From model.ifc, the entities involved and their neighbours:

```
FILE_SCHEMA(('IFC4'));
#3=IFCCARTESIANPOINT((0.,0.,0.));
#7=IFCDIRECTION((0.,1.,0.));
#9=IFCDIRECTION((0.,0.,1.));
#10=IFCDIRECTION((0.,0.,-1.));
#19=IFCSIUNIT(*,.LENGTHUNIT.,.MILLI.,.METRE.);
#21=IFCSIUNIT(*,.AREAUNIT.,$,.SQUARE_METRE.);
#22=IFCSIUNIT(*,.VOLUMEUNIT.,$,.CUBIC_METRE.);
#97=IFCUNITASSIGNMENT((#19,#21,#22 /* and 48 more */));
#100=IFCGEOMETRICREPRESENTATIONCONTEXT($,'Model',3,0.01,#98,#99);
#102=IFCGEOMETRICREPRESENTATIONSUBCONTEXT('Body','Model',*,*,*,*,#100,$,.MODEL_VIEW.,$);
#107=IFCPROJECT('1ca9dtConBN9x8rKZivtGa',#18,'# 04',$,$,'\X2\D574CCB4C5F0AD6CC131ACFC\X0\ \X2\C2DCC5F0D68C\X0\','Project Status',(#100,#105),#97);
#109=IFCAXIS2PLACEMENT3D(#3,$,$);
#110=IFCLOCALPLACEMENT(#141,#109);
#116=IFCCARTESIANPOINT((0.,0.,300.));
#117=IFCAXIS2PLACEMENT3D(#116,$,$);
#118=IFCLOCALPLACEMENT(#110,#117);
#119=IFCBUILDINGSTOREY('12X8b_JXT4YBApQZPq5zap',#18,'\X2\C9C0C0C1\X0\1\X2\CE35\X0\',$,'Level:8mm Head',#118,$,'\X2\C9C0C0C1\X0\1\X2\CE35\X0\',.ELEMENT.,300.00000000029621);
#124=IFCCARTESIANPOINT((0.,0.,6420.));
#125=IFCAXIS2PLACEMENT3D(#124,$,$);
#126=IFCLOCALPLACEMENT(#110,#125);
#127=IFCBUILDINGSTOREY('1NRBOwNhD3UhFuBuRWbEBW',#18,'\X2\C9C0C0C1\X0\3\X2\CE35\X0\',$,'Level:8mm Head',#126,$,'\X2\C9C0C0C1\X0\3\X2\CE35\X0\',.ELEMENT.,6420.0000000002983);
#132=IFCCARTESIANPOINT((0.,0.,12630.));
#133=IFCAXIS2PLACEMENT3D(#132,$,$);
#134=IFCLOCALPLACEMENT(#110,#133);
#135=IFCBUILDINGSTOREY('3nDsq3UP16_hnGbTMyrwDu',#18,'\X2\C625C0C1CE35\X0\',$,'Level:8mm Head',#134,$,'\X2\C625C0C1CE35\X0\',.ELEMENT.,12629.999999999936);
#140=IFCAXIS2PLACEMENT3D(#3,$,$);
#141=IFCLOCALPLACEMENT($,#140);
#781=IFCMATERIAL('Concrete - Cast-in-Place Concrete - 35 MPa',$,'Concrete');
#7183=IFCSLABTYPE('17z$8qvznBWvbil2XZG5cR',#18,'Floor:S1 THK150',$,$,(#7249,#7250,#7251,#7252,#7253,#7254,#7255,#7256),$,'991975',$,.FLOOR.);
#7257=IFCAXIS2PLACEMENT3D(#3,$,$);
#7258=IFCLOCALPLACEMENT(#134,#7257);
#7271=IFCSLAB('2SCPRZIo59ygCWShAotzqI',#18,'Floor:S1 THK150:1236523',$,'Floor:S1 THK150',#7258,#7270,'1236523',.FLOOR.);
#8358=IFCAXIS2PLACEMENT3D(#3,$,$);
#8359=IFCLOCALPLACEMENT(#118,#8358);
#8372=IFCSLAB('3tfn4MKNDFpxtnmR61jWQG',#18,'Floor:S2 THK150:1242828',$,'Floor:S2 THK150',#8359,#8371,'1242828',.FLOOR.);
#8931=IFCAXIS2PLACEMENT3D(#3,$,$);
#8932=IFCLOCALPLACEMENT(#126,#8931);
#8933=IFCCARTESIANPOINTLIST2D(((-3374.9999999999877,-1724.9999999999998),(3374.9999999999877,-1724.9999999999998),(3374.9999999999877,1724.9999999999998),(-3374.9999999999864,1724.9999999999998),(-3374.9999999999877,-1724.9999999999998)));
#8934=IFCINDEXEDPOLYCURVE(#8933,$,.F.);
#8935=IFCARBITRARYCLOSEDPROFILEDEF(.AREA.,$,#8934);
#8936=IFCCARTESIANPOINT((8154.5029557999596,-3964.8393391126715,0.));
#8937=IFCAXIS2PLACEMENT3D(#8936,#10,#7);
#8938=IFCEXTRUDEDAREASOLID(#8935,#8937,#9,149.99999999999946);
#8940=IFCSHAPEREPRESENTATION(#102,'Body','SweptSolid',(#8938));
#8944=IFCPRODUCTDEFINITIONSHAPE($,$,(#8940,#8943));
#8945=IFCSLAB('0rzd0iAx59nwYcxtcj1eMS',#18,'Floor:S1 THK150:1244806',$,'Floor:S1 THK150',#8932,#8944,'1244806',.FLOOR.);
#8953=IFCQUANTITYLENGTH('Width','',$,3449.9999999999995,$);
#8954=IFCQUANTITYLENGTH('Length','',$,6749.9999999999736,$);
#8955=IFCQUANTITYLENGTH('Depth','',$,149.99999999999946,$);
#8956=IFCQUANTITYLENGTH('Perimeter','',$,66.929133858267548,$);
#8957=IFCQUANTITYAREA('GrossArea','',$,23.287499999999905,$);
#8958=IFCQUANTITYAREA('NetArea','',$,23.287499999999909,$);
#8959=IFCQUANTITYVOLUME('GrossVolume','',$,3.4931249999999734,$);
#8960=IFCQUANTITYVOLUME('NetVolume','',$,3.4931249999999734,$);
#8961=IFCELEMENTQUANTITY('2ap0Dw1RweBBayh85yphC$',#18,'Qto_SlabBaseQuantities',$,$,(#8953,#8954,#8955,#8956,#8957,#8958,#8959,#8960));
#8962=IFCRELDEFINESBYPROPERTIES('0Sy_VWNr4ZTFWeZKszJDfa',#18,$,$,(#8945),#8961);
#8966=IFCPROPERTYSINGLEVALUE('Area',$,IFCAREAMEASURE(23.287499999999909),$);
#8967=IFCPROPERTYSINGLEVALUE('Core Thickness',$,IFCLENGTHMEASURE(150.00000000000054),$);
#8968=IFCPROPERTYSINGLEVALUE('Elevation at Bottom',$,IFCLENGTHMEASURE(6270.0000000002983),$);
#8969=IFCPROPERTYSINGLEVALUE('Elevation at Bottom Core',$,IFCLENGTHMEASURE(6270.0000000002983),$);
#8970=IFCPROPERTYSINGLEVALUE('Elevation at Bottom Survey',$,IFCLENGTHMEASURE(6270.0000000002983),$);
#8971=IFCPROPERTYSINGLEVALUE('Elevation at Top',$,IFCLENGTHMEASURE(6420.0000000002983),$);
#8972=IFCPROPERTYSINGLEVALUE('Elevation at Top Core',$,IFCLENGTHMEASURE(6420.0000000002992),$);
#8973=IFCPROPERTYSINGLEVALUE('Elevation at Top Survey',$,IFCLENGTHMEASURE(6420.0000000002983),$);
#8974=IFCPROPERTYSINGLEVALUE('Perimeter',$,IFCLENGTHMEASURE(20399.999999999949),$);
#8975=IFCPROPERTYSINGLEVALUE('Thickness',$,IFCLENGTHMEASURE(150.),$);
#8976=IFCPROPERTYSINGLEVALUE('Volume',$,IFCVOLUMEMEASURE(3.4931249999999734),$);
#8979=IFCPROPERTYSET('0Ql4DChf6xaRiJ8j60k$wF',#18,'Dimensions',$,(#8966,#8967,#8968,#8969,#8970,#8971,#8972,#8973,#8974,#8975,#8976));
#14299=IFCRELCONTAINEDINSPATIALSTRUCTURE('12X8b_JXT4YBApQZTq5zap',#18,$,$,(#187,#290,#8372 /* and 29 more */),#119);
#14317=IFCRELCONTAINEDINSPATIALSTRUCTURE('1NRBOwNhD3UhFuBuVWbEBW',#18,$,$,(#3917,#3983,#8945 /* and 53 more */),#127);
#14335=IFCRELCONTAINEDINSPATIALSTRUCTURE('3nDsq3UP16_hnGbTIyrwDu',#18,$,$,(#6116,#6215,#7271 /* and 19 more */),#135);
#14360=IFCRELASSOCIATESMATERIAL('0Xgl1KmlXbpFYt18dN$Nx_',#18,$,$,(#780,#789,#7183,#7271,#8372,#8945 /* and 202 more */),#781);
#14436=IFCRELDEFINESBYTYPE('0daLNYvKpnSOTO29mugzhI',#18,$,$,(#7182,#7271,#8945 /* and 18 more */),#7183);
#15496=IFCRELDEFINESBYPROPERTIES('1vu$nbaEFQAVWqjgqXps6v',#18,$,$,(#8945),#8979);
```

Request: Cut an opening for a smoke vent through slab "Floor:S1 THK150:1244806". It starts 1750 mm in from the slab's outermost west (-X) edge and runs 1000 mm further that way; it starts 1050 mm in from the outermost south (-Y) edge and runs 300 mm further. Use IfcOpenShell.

```python
import numpy as np
import ifcopenshell
import ifcopenshell.api.feature
import ifcopenshell.api.geometry
import ifcopenshell.api.pset
import ifcopenshell.api.root
import ifcopenshell.geom
import ifcopenshell.util.element
import ifcopenshell.util.placement
import ifcopenshell.util.representation
import ifcopenshell.util.shape
import ifcopenshell.util.unit

model = ifcopenshell.open("model.ifc")
unit_scale = ifcopenshell.util.unit.calculate_unit_scale(model)
area_scale = ifcopenshell.util.unit.calculate_unit_scale(model, "AREAUNIT")
volume_scale = ifcopenshell.util.unit.calculate_unit_scale(model, "VOLUMEUNIT")
settings = ifcopenshell.geom.settings()


def volume(element):
    """Net volume in cubic metres, openings subtracted."""
    shape = ifcopenshell.geom.create_shape(settings, element)
    return ifcopenshell.util.shape.get_volume(shape.geometry)


slab = model.by_guid("0rzd0iAx59nwYcxtcj1eMS")
before = volume(slab)

# Extent in the slab's own axes, in metres. The edges named are its -X and -Y sides.
slab_shape = ifcopenshell.geom.create_shape(settings, slab)
vertices = ifcopenshell.util.shape.get_vertices(slab_shape.geometry)
x_min, y_min, bottom = vertices.min(axis=0)
top = vertices[:, 2].max()

opening = ifcopenshell.api.root.create_entity(model, ifc_class="IfcOpeningElement", name="Smoke vent opening", predefined_type="OPENING")
context = ifcopenshell.util.representation.get_context(model, "Model", "Body", "MODEL_VIEW")
width, depth = 1, 0.3
outline = [(0.0, 0.0), (width, 0.0), (width, depth), (0.0, depth), (0.0, 0.0)]
# Overshoot both faces by 50 mm so the cut is clean.
shape = ifcopenshell.api.geometry.add_slab_representation(
    model, context=context, depth=top - bottom + 0.1, polyline=outline
)
ifcopenshell.api.geometry.assign_representation(model, product=opening, representation=shape)

matrix = ifcopenshell.util.placement.get_local_placement(slab.ObjectPlacement)
matrix[:, 3] = matrix @ np.append(np.array([x_min + 1.75, y_min + 1.05, bottom - 0.05]) / unit_scale, 1.0)
ifcopenshell.api.geometry.edit_object_placement(model, product=opening, matrix=matrix, is_si=False)
ifcopenshell.api.feature.add_feature(model, feature=opening, element=slab)

after = volume(slab)

# Update the slab's stored quantities.
qto = model.by_id(ifcopenshell.util.element.get_pset(slab, "Qto_SlabBaseQuantities", should_inherit=False)["id"])
ifcopenshell.api.pset.edit_qto(model, qto=qto, properties={
    "NetArea": after / (top - bottom) / area_scale,
    "NetVolume": after / volume_scale,
})
pset = model.by_id(ifcopenshell.util.element.get_pset(slab, "Dimensions", should_inherit=False)["id"])
ifcopenshell.api.pset.edit_pset(model, pset=pset, properties={
    "Area": model.create_entity("IfcAreaMeasure", after / (top - bottom) / area_scale),
    "Volume": model.create_entity("IfcVolumeMeasure", after / volume_scale),
})

print(f"slab volume {before:.3f} -> {after:.3f} m3")

model.write("model_rev.ifc")
```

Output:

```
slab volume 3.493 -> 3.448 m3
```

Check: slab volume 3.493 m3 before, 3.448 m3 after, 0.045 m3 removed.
